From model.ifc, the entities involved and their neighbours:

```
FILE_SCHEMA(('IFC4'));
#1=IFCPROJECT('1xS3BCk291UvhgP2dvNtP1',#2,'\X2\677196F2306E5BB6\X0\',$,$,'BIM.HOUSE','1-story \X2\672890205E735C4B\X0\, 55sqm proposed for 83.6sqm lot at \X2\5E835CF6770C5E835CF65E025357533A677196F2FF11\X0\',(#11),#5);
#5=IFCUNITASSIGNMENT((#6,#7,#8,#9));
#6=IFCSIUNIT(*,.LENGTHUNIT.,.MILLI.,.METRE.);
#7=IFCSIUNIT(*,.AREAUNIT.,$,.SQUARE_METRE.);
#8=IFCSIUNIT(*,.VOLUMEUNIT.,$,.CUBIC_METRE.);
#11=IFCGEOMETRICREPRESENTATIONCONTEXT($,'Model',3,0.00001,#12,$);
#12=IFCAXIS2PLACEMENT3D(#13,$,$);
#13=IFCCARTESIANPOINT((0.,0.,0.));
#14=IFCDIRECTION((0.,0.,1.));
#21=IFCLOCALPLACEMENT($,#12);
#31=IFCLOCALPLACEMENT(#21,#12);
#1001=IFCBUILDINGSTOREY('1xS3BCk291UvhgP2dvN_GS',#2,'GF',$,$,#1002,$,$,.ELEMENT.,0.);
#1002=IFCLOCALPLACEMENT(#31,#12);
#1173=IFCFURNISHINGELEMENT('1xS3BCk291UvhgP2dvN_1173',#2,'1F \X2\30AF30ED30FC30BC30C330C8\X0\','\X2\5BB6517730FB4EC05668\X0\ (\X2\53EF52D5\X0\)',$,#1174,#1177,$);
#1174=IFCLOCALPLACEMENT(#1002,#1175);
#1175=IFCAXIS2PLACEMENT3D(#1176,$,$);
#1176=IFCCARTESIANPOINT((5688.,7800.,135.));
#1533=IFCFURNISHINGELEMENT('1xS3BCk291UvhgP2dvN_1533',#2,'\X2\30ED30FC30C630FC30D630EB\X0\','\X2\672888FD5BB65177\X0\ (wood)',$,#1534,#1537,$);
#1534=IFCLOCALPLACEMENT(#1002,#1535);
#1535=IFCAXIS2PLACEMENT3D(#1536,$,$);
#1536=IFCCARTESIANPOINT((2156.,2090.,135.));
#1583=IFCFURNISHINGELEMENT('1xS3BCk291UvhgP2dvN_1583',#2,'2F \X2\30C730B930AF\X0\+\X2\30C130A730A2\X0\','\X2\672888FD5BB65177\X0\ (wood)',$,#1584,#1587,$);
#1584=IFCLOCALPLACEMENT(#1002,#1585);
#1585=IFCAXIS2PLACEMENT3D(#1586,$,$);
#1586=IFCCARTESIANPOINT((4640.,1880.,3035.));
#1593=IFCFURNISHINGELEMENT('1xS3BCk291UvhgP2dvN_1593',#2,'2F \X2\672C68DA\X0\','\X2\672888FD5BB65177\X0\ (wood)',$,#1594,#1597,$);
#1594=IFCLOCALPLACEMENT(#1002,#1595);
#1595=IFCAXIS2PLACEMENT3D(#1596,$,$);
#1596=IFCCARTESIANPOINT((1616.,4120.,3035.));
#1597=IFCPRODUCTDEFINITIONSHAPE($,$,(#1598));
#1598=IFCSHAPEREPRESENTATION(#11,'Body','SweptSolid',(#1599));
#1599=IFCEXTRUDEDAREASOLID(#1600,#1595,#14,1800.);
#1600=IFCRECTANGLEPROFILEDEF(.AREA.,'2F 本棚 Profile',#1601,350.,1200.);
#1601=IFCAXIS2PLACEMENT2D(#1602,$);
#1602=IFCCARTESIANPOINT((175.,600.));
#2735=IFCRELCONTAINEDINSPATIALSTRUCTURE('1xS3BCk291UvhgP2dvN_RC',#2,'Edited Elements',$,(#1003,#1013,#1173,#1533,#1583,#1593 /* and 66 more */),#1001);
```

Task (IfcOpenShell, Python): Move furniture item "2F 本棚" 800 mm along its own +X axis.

```python
import ifcopenshell
import ifcopenshell.api.geometry
import ifcopenshell.util.placement

model = ifcopenshell.open("model.ifc")

item = model.by_guid("1xS3BCk291UvhgP2dvN_1593")
matrix = ifcopenshell.util.placement.get_local_placement(item.ObjectPlacement)
matrix[:3, 3] += matrix[:3, 0] * 800.0
ifcopenshell.api.geometry.edit_object_placement(model, product=item, matrix=matrix, is_si=False)

print(ifcopenshell.util.placement.get_local_placement(item.ObjectPlacement).round(3) + 0.0)

model.write("model_edited.ifc")
```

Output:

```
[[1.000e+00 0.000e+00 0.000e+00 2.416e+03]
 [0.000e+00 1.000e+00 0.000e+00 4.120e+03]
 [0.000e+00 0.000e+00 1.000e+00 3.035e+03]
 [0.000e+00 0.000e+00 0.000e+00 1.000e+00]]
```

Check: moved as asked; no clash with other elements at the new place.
